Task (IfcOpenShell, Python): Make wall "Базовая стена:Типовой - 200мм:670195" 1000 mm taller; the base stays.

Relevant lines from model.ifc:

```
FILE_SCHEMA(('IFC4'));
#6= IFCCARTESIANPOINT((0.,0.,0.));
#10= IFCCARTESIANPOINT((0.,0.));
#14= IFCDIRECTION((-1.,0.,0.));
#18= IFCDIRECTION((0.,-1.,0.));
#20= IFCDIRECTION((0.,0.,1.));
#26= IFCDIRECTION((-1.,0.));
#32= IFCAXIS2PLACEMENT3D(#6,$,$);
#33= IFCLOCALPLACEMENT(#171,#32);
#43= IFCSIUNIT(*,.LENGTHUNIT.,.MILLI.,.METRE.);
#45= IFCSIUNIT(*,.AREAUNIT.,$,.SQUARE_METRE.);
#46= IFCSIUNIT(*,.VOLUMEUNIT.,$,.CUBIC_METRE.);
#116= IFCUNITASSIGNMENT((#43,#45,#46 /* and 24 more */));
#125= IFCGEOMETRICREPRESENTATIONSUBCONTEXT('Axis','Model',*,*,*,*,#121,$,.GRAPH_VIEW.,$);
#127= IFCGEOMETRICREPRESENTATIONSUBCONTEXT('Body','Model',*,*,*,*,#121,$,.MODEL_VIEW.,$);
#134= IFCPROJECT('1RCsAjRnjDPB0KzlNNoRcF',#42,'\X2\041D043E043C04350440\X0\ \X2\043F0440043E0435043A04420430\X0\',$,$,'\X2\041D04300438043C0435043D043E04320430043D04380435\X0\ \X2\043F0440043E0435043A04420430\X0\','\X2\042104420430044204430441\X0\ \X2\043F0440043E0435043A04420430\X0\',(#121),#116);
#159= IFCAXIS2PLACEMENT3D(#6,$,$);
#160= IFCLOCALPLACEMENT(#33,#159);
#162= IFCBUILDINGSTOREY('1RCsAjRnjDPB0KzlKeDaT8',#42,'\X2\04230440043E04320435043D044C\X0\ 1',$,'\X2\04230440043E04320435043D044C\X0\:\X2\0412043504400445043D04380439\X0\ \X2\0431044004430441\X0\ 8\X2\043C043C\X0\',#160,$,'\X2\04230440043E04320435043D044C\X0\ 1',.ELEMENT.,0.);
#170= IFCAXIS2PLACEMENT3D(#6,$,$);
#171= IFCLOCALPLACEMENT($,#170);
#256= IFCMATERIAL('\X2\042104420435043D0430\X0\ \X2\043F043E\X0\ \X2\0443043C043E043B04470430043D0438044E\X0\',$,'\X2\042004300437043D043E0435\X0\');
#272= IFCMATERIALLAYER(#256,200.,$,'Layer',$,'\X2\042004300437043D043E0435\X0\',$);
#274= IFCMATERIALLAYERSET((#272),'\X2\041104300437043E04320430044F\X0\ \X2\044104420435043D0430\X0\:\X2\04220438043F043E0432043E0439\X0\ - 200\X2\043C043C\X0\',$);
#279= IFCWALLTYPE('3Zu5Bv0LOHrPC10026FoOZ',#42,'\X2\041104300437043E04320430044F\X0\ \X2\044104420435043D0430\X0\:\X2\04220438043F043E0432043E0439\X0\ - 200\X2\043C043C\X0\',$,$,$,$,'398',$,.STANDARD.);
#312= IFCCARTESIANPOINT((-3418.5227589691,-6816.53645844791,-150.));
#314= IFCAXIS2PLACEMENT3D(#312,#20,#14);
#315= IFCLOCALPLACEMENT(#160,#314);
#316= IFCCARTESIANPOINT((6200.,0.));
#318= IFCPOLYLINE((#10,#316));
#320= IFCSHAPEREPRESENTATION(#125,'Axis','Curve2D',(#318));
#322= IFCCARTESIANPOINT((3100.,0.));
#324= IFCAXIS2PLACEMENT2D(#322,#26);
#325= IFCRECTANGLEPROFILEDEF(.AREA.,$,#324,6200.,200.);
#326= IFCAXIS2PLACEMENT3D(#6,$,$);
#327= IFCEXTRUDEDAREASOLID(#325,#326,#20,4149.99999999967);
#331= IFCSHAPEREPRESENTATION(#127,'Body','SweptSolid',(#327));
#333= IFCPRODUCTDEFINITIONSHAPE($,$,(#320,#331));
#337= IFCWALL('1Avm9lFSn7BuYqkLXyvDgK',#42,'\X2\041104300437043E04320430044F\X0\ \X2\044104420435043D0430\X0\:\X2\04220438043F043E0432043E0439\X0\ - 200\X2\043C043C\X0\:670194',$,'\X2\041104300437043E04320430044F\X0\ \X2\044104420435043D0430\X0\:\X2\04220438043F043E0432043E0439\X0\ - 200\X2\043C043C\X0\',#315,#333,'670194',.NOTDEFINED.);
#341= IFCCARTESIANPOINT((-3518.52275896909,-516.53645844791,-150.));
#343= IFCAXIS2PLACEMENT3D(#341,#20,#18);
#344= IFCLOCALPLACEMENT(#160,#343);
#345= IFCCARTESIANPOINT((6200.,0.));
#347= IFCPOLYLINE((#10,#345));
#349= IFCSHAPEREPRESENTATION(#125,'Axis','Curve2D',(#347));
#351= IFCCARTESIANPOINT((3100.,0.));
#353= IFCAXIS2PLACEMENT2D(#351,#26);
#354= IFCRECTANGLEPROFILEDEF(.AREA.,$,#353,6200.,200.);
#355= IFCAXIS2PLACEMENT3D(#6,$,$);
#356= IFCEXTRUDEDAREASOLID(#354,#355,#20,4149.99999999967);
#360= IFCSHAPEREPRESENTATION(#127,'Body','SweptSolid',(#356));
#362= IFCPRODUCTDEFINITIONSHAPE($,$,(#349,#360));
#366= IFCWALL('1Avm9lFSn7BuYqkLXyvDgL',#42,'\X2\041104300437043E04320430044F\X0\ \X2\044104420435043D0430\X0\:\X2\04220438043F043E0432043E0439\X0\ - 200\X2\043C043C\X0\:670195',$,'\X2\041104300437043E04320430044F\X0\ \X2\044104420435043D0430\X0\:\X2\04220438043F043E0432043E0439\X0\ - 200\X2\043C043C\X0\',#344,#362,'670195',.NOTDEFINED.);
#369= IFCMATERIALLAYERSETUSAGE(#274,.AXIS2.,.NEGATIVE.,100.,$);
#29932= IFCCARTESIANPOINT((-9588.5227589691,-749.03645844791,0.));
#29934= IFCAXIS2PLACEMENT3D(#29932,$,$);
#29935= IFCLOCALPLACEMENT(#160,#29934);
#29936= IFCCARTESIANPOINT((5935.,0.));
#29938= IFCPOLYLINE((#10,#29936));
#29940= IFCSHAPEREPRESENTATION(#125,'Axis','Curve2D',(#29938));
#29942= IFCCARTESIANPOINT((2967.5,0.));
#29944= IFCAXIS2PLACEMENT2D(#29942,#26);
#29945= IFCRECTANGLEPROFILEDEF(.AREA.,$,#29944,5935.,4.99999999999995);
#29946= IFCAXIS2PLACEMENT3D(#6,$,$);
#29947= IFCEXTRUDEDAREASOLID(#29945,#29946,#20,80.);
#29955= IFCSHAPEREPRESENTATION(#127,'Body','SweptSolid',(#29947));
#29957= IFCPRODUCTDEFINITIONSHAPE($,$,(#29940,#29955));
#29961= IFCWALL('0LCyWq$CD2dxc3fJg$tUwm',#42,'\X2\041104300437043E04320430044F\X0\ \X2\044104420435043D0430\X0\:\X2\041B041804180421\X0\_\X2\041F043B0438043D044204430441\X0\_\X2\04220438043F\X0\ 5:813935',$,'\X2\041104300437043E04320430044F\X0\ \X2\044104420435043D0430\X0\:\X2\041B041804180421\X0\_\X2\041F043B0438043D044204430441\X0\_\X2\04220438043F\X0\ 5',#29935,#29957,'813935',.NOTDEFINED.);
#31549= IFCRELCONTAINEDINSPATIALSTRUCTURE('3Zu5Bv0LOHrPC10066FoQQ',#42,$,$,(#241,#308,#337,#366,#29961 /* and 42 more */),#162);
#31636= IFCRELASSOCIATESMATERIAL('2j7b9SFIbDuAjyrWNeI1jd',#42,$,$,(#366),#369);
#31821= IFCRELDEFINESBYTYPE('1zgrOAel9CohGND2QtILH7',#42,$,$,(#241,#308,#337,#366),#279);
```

```python
import ifcopenshell
import ifcopenshell.geom
import ifcopenshell.util.representation
import ifcopenshell.util.shape

model = ifcopenshell.open("model.ifc")
settings = ifcopenshell.geom.settings()


def volume(element):
    """Net volume in cubic metres, openings subtracted."""
    shape = ifcopenshell.geom.create_shape(settings, element)
    return ifcopenshell.util.shape.get_volume(shape.geometry)


wall = model.by_guid("1Avm9lFSn7BuYqkLXyvDgL")
before = volume(wall)

body = ifcopenshell.util.representation.get_representation(wall, "Model", "Body")
solid = body.Items[0]
old_height = solid.Depth
solid.Depth += 1000.0
after = volume(wall)

print(f"height {old_height:g} -> {solid.Depth:g}, volume {before:.3f} -> {after:.3f} m3")

model.write("model_edited.ifc")
```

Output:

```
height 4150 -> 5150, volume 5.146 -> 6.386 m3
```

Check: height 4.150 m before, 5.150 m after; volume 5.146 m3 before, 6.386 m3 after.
